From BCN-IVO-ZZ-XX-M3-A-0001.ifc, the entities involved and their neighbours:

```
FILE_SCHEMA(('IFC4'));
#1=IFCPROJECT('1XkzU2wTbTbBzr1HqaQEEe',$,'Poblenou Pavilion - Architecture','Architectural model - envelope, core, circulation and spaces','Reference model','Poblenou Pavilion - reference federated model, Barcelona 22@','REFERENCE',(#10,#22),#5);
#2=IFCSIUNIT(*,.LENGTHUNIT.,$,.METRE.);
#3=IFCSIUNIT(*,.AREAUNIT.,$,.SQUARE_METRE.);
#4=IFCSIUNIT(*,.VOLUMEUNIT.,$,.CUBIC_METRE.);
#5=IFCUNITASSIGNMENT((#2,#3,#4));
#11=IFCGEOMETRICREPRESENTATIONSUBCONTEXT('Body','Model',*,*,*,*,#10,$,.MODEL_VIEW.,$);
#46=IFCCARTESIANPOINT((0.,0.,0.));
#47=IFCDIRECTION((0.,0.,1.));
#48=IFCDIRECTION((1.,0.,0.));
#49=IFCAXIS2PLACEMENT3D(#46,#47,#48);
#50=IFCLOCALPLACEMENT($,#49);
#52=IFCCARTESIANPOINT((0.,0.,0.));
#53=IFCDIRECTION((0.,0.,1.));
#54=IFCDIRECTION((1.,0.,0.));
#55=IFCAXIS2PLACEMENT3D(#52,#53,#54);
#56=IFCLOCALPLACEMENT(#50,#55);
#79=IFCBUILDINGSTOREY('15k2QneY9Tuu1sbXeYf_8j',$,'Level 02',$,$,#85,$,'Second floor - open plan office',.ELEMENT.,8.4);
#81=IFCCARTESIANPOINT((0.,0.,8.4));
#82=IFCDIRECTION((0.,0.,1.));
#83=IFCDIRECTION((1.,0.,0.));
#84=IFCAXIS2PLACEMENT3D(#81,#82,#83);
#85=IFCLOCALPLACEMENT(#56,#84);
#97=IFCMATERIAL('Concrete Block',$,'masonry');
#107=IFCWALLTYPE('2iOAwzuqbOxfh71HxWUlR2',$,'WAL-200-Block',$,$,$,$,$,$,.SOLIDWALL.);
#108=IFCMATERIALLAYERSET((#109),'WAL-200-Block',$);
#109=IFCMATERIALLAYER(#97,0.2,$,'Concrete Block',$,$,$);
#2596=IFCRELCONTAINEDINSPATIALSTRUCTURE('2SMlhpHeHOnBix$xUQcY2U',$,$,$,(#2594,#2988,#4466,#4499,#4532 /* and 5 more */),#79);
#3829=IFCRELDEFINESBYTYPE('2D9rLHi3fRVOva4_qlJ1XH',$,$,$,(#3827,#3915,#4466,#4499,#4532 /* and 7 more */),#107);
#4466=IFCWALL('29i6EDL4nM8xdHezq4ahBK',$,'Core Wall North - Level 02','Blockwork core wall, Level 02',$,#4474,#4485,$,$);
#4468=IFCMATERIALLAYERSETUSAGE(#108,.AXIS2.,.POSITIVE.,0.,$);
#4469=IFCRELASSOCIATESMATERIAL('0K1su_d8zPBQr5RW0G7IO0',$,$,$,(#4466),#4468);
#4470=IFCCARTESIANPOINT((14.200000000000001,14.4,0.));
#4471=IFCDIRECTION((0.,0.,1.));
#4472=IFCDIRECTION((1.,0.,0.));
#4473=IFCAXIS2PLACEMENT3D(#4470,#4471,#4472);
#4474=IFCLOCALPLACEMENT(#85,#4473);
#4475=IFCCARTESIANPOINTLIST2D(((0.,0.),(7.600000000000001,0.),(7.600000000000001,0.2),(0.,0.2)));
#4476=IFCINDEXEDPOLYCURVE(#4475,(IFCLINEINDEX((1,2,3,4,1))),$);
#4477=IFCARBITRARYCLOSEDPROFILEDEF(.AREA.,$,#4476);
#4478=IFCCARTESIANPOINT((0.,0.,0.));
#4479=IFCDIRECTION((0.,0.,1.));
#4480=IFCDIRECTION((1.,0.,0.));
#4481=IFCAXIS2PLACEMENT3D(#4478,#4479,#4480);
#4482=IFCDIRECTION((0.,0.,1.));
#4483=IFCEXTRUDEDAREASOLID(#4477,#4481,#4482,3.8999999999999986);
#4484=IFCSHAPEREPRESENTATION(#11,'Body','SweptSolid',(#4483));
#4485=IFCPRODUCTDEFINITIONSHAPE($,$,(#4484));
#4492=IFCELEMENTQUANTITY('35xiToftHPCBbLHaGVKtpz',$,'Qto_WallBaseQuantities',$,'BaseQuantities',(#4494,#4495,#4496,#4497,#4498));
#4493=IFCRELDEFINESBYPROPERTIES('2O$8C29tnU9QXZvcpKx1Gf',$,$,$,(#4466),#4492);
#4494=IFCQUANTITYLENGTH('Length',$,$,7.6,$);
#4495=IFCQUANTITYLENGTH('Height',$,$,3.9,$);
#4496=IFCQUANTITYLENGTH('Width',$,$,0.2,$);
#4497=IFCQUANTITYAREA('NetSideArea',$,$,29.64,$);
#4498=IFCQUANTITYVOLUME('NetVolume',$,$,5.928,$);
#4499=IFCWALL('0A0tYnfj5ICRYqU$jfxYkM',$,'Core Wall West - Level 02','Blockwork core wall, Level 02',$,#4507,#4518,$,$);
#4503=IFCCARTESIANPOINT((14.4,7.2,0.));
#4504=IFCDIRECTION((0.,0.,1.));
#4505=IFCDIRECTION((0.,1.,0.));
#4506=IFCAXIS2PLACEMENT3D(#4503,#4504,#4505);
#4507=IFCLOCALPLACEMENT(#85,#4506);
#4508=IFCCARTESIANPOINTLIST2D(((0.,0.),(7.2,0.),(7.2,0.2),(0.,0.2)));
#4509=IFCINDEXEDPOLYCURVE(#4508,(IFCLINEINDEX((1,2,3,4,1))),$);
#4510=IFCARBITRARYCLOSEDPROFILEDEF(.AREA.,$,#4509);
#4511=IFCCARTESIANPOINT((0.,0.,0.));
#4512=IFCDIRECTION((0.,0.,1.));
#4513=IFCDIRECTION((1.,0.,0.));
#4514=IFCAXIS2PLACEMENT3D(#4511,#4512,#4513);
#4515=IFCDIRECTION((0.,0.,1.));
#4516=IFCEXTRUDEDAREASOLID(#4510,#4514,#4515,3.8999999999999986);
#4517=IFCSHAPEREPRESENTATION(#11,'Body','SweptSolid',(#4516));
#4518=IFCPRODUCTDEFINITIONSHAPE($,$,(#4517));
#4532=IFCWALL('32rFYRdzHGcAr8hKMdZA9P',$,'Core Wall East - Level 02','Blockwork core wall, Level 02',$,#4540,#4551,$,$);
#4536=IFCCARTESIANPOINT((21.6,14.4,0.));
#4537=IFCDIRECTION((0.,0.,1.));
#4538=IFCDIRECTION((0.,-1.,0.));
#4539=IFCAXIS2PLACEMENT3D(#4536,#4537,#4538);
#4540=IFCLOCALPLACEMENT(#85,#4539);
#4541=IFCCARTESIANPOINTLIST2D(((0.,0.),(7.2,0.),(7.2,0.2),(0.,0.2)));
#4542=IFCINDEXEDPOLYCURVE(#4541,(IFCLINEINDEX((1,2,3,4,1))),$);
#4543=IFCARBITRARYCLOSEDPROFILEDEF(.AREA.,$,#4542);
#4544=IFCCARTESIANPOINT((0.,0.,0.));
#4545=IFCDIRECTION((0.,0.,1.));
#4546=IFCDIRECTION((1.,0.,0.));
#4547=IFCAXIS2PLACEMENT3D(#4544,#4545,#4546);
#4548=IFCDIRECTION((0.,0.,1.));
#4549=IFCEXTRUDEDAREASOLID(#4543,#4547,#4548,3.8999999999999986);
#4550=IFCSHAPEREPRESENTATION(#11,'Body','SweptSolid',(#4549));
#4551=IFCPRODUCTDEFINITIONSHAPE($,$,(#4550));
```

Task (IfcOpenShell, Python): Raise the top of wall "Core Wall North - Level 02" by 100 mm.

```python
import ifcopenshell
import ifcopenshell.api.pset
import ifcopenshell.geom
import ifcopenshell.util.element
import ifcopenshell.util.representation
import ifcopenshell.util.shape
import ifcopenshell.util.unit

model = ifcopenshell.open("BCN-IVO-ZZ-XX-M3-A-0001.ifc")
area_scale = ifcopenshell.util.unit.calculate_unit_scale(model, "AREAUNIT")
volume_scale = ifcopenshell.util.unit.calculate_unit_scale(model, "VOLUMEUNIT")
settings = ifcopenshell.geom.settings()


def volume(element):
    """Net volume in cubic metres, openings subtracted."""
    shape = ifcopenshell.geom.create_shape(settings, element)
    return ifcopenshell.util.shape.get_volume(shape.geometry)


wall = model.by_guid("29i6EDL4nM8xdHezq4ahBK")
before = volume(wall)

body = ifcopenshell.util.representation.get_representation(wall, "Model", "Body")
solid = body.Items[0]
old_height = solid.Depth
solid.Depth += 0.1
after = volume(wall)
thickness = 0.2  # wall thickness in metres

# Update the stored height, areas and volumes.
qto = model.by_id(ifcopenshell.util.element.get_pset(wall, "Qto_WallBaseQuantities", should_inherit=False)["id"])
ifcopenshell.api.pset.edit_qto(model, qto=qto, properties={
    "Height": solid.Depth,
    "NetSideArea": after / thickness / area_scale,
    "NetVolume": after / volume_scale,
})

print(f"height {old_height:g} -> {solid.Depth:g}, volume {before:.3f} -> {after:.3f} m3")

model.write("BCN-IVO-ZZ-XX-M3-A-0001_v2.ifc")
```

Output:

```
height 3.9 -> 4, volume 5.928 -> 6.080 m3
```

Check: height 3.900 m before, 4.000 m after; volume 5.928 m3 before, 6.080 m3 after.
